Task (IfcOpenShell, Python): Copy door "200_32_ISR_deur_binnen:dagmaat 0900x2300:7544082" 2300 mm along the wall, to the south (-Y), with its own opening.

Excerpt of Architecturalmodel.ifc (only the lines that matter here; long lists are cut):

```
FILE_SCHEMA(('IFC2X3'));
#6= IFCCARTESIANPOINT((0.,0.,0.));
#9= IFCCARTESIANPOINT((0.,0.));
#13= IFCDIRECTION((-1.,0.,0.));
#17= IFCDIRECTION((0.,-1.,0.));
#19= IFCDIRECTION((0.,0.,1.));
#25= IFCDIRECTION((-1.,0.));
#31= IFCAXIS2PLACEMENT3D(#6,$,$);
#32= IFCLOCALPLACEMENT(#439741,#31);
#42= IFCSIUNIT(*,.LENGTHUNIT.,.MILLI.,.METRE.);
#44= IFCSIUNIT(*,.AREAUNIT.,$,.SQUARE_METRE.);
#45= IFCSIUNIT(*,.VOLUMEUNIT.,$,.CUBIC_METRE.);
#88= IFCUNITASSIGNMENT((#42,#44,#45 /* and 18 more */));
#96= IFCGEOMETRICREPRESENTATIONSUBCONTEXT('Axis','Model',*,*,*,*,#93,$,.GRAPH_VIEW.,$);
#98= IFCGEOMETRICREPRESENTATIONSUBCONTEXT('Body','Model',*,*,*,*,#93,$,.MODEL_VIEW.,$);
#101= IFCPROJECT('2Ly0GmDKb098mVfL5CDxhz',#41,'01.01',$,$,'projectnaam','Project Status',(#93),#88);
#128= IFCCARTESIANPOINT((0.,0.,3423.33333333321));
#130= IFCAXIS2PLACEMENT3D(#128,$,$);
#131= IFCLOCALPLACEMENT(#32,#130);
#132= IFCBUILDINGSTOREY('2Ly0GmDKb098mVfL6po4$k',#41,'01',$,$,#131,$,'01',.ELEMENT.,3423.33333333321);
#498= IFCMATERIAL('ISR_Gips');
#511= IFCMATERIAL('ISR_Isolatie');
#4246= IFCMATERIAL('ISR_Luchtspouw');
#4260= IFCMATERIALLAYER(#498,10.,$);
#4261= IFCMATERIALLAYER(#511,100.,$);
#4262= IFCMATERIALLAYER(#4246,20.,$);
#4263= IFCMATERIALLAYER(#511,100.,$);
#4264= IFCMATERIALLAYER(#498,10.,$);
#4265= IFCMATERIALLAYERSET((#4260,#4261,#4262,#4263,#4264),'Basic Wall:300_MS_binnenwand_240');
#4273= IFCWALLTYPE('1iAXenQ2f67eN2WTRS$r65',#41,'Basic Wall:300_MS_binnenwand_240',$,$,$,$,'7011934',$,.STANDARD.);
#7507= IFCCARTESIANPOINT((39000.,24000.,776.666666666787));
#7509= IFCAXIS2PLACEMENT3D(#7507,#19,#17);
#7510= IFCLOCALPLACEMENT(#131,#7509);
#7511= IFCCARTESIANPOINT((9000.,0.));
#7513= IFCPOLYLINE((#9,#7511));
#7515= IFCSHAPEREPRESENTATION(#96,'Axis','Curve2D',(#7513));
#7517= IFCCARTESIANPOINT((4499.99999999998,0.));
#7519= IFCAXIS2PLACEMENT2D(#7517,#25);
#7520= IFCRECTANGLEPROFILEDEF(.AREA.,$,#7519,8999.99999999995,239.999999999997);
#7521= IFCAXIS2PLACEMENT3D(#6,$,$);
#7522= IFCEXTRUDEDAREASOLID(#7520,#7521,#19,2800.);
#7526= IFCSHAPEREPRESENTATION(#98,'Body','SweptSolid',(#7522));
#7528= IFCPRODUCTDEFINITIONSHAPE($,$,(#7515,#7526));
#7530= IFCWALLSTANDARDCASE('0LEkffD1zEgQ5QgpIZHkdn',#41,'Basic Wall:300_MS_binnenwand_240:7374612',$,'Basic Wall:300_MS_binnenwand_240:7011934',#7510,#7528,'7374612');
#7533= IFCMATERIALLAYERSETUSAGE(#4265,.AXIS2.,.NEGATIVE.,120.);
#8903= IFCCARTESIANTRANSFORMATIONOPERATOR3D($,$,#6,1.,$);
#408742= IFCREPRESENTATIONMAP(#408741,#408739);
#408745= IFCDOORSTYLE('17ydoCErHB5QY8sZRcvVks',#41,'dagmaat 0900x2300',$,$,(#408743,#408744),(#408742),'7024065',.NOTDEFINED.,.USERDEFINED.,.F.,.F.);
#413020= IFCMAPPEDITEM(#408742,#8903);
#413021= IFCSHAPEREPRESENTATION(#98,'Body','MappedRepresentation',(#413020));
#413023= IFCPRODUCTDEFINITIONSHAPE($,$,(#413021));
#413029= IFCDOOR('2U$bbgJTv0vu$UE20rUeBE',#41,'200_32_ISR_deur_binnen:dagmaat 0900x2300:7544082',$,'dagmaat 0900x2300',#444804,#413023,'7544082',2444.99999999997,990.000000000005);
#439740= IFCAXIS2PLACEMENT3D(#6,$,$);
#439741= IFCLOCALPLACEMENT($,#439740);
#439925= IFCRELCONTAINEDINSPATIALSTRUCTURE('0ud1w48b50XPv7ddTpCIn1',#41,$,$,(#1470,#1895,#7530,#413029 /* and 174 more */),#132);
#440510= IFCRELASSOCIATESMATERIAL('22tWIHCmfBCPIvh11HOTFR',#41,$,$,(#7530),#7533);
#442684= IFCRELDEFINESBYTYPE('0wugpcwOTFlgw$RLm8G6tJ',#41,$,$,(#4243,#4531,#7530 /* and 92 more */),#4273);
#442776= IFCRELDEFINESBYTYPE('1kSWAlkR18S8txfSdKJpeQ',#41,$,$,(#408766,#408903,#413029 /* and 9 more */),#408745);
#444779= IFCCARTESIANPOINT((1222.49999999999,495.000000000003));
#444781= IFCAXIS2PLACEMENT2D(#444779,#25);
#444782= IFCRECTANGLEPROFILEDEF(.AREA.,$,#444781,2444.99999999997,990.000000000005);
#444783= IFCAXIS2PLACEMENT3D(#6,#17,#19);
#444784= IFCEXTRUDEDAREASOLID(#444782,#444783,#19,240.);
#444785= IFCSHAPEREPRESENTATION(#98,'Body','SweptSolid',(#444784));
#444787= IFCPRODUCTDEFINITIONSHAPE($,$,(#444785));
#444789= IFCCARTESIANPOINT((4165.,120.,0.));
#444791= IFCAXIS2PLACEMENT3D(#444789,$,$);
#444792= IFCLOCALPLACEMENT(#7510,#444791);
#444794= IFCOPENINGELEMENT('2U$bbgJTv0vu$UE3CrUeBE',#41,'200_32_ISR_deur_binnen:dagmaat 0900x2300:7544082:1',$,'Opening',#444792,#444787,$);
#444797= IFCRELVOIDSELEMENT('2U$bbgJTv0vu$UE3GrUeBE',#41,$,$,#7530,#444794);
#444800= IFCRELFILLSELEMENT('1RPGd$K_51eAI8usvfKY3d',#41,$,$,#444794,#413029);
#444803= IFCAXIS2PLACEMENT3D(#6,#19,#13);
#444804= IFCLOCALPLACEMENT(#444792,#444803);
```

```python
import ifcopenshell
import ifcopenshell.api.feature
import ifcopenshell.api.geometry
import ifcopenshell.api.root
import ifcopenshell.geom
import ifcopenshell.util.element
import ifcopenshell.util.placement
import ifcopenshell.util.shape
import ifcopenshell.util.unit

model = ifcopenshell.open("Architecturalmodel.ifc")
unit_scale = ifcopenshell.util.unit.calculate_unit_scale(model)
settings = ifcopenshell.geom.settings()


def volume(element):
    """Net volume in cubic metres, openings subtracted."""
    shape = ifcopenshell.geom.create_shape(settings, element)
    return ifcopenshell.util.shape.get_volume(shape.geometry)


def reuse_history(source, copy):
    """copy_class also copies each property set's owner history, people and application; keep the originals."""
    for rel in copy.IsDefinedBy:
        if rel.is_a("IfcRelDefinesByProperties") and (history := rel.RelatingPropertyDefinition.OwnerHistory):
            rel.RelatingPropertyDefinition.OwnerHistory = source.OwnerHistory
            ifcopenshell.util.element.remove_deep2(model, history)


door = model.by_guid("2U$bbgJTv0vu$UE20rUeBE")
opening = door.FillsVoids[0].RelatingOpeningElement
wall = opening.VoidsElements[0].RelatingBuildingElement
before = volume(wall)
shift = ifcopenshell.util.placement.get_local_placement(wall.ObjectPlacement)[:3, 0] * 2.3 / unit_scale

# copy_class copies the void relationship, type, container and properties, but no geometry.
new_opening = ifcopenshell.api.root.copy_class(model, product=opening)
new_opening.Representation = ifcopenshell.util.element.copy_deep(
    model, opening.Representation, exclude=["IfcGeometricRepresentationContext", "IfcRepresentationMap"]
)
new_opening.Name = "200_32_ISR_deur_binnen:dagmaat 0900x2300"
new_door = ifcopenshell.api.root.copy_class(model, product=door)
new_door.Representation = ifcopenshell.util.element.copy_deep(
    model, door.Representation, exclude=["IfcGeometricRepresentationContext", "IfcRepresentationMap"]
)
new_door.Name = "200_32_ISR_deur_binnen:dagmaat 0900x2300"
new_door.Tag = None
reuse_history(door, new_door)
fills = ifcopenshell.api.feature.add_filling(model, opening=new_opening, element=new_door)
fills.OwnerHistory = new_door.OwnerHistory  # required in IFC2X3

for old, new in ((opening, new_opening), (door, new_door)):
    matrix = ifcopenshell.util.placement.get_local_placement(old.ObjectPlacement)
    matrix[:3, 3] += shift
    ifcopenshell.api.geometry.edit_object_placement(model, product=new, matrix=matrix, is_si=False)

after = volume(wall)

print(f"wall volume {before:.3f} -> {after:.3f} m3")

model.write("Architecturalmodel-out.ifc")
```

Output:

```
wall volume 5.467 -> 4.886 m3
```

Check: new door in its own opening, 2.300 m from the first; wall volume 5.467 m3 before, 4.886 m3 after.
